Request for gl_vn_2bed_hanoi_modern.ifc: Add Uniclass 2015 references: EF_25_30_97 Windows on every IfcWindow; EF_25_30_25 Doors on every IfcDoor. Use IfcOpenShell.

First a look at what the model holds.

```python
import ifcopenshell

model = ifcopenshell.open("gl_vn_2bed_hanoi_modern.ifc")
print(model.schema)
print("classifications:", [c.Name for c in model.by_type("IfcClassification")])
for ifc_class in ("IfcDoor", "IfcRoof", "IfcStair", "IfcWall", "IfcWindow"):
    print(ifc_class, len(model.by_type(ifc_class)))
```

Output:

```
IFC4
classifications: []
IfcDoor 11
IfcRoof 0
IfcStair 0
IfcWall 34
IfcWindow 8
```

```python
import ifcopenshell
import ifcopenshell.api.classification

model = ifcopenshell.open("gl_vn_2bed_hanoi_modern.ifc")

system = ifcopenshell.api.classification.add_classification(model, classification="Uniclass 2015")

codes = {
    "IfcWindow": ("EF_25_30_97", "Windows"),
    "IfcDoor": ("EF_25_30_25", "Doors"),
}
for ifc_class, (code, name) in codes.items():
    products = model.by_type(ifc_class)
    ifcopenshell.api.classification.add_reference(
        model, products=products, classification=system, identification=code, name=name
    )
    print(code, len(products))

model.write("gl_vn_2bed_hanoi_modern_rev.ifc")
```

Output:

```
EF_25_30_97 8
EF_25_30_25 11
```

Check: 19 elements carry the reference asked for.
